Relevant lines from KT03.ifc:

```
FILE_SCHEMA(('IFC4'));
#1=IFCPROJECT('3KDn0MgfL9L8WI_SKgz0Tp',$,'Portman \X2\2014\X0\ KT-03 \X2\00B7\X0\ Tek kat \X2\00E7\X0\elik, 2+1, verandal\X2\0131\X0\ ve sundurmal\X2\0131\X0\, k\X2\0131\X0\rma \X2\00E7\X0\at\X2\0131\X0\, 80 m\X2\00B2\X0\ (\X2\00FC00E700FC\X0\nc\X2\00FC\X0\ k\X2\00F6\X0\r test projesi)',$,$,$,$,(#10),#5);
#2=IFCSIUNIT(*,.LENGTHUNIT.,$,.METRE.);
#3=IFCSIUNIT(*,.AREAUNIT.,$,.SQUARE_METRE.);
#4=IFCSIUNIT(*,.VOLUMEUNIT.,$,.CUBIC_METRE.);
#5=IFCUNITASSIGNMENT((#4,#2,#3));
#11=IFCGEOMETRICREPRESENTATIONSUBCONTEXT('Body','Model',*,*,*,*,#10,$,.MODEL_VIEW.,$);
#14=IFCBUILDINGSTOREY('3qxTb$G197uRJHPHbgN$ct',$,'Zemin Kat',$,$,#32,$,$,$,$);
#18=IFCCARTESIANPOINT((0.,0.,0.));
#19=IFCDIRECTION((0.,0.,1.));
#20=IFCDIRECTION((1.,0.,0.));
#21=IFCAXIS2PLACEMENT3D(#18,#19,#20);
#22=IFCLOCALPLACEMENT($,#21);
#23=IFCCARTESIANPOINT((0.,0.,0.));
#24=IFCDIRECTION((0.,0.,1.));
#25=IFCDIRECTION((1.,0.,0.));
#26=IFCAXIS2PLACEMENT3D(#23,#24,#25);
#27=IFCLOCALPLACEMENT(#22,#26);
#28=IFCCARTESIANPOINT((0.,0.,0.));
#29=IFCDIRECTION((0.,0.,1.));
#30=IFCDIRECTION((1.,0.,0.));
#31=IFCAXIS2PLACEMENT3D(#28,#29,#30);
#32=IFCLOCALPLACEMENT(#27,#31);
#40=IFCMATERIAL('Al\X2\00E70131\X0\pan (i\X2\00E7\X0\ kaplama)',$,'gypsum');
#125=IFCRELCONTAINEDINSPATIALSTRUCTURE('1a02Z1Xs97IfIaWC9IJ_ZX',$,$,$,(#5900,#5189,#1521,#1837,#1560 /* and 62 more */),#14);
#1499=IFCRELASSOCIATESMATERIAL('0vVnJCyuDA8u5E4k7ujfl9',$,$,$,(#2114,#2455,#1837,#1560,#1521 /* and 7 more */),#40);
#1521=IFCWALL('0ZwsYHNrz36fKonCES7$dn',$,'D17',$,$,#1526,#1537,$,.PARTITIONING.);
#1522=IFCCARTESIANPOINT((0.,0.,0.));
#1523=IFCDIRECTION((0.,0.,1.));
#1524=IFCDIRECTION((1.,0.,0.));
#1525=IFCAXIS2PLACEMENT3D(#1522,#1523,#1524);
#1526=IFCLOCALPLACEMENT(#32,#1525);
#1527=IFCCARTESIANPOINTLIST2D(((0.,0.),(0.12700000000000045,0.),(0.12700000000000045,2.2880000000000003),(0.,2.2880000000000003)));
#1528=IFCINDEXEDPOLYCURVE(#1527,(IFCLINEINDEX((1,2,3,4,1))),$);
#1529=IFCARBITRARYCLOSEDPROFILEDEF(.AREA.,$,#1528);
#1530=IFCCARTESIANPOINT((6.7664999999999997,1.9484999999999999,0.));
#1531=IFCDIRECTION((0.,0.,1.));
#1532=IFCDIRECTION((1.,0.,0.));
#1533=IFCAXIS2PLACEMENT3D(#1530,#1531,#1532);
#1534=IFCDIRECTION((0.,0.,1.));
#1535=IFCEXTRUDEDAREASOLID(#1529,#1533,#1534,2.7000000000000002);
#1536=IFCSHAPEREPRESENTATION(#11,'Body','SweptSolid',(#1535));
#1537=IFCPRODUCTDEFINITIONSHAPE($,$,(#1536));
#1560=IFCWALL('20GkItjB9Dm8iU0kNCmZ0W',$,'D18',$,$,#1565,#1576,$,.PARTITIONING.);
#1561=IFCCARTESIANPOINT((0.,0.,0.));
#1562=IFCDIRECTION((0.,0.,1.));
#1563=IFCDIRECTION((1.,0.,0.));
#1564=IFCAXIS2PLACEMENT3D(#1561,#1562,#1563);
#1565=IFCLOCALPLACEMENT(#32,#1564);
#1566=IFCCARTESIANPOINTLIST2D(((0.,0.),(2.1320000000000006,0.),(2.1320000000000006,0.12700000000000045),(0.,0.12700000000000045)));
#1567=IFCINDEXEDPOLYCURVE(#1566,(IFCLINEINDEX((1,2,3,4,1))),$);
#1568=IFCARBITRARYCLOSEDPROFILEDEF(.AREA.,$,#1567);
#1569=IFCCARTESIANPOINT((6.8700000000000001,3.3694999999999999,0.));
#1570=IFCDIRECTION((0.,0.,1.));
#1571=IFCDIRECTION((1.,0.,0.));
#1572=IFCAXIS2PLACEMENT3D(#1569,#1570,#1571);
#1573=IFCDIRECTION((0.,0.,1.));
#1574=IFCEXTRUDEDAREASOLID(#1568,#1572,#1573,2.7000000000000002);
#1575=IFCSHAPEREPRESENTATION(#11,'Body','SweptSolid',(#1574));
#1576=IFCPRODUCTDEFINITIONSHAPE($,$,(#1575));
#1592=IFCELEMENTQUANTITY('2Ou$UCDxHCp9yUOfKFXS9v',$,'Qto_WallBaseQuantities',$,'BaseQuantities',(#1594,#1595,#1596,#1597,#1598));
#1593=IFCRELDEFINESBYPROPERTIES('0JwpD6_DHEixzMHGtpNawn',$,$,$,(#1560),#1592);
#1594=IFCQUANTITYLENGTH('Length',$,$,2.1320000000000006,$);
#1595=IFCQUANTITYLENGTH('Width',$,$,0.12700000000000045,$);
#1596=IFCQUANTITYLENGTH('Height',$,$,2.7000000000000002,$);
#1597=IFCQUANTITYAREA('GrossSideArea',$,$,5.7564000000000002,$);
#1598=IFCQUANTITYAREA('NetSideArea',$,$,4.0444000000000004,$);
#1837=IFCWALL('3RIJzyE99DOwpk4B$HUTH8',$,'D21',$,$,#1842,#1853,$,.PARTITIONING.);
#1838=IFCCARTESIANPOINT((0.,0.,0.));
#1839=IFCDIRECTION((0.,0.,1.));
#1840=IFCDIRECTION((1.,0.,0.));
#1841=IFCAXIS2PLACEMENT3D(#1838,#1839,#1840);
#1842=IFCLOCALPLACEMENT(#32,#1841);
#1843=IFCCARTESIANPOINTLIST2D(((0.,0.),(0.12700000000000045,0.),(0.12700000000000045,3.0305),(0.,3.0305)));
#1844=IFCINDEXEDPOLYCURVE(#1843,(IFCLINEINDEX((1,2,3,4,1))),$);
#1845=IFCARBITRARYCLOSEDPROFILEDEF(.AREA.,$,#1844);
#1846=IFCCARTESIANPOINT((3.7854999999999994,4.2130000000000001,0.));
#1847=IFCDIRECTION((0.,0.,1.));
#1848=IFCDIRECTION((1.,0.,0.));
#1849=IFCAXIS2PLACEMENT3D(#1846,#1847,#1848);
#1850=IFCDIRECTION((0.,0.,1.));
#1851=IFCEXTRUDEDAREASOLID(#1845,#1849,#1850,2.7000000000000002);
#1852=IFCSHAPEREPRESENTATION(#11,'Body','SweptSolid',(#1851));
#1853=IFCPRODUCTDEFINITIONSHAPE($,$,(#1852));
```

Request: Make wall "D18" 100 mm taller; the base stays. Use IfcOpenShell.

```python
import ifcopenshell
import ifcopenshell.api.pset
import ifcopenshell.geom
import ifcopenshell.util.element
import ifcopenshell.util.representation
import ifcopenshell.util.shape
import ifcopenshell.util.unit

model = ifcopenshell.open("KT03.ifc")
unit_scale = ifcopenshell.util.unit.calculate_unit_scale(model)
area_scale = ifcopenshell.util.unit.calculate_unit_scale(model, "AREAUNIT")
settings = ifcopenshell.geom.settings()


def volume(element):
    """Net volume in cubic metres, openings subtracted."""
    shape = ifcopenshell.geom.create_shape(settings, element)
    return ifcopenshell.util.shape.get_volume(shape.geometry)


wall = model.by_id(1560)
before = volume(wall)

body = ifcopenshell.util.representation.get_representation(wall, "Model", "Body")
solid = body.Items[0]
old_height = solid.Depth
solid.Depth += 0.1 / unit_scale
after = volume(wall)
thickness = 0.127  # wall thickness in metres

# Update the stored height, areas and volumes.
qto = model.by_id(ifcopenshell.util.element.get_pset(wall, "Qto_WallBaseQuantities", should_inherit=False)["id"])
ifcopenshell.api.pset.edit_qto(model, qto=qto, properties={
    "Height": solid.Depth,
    "GrossSideArea": ifcopenshell.util.element.get_pset(wall, "Qto_WallBaseQuantities", "GrossSideArea") * solid.Depth / old_height,
    "NetSideArea": after / thickness / area_scale,
})

print(f"height {old_height:g} -> {solid.Depth:g}, volume {before:.3f} -> {after:.3f} m3")

model.write("KT03_rev.ifc")
```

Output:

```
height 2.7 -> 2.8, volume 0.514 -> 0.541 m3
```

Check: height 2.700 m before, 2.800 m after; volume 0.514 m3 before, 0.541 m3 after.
